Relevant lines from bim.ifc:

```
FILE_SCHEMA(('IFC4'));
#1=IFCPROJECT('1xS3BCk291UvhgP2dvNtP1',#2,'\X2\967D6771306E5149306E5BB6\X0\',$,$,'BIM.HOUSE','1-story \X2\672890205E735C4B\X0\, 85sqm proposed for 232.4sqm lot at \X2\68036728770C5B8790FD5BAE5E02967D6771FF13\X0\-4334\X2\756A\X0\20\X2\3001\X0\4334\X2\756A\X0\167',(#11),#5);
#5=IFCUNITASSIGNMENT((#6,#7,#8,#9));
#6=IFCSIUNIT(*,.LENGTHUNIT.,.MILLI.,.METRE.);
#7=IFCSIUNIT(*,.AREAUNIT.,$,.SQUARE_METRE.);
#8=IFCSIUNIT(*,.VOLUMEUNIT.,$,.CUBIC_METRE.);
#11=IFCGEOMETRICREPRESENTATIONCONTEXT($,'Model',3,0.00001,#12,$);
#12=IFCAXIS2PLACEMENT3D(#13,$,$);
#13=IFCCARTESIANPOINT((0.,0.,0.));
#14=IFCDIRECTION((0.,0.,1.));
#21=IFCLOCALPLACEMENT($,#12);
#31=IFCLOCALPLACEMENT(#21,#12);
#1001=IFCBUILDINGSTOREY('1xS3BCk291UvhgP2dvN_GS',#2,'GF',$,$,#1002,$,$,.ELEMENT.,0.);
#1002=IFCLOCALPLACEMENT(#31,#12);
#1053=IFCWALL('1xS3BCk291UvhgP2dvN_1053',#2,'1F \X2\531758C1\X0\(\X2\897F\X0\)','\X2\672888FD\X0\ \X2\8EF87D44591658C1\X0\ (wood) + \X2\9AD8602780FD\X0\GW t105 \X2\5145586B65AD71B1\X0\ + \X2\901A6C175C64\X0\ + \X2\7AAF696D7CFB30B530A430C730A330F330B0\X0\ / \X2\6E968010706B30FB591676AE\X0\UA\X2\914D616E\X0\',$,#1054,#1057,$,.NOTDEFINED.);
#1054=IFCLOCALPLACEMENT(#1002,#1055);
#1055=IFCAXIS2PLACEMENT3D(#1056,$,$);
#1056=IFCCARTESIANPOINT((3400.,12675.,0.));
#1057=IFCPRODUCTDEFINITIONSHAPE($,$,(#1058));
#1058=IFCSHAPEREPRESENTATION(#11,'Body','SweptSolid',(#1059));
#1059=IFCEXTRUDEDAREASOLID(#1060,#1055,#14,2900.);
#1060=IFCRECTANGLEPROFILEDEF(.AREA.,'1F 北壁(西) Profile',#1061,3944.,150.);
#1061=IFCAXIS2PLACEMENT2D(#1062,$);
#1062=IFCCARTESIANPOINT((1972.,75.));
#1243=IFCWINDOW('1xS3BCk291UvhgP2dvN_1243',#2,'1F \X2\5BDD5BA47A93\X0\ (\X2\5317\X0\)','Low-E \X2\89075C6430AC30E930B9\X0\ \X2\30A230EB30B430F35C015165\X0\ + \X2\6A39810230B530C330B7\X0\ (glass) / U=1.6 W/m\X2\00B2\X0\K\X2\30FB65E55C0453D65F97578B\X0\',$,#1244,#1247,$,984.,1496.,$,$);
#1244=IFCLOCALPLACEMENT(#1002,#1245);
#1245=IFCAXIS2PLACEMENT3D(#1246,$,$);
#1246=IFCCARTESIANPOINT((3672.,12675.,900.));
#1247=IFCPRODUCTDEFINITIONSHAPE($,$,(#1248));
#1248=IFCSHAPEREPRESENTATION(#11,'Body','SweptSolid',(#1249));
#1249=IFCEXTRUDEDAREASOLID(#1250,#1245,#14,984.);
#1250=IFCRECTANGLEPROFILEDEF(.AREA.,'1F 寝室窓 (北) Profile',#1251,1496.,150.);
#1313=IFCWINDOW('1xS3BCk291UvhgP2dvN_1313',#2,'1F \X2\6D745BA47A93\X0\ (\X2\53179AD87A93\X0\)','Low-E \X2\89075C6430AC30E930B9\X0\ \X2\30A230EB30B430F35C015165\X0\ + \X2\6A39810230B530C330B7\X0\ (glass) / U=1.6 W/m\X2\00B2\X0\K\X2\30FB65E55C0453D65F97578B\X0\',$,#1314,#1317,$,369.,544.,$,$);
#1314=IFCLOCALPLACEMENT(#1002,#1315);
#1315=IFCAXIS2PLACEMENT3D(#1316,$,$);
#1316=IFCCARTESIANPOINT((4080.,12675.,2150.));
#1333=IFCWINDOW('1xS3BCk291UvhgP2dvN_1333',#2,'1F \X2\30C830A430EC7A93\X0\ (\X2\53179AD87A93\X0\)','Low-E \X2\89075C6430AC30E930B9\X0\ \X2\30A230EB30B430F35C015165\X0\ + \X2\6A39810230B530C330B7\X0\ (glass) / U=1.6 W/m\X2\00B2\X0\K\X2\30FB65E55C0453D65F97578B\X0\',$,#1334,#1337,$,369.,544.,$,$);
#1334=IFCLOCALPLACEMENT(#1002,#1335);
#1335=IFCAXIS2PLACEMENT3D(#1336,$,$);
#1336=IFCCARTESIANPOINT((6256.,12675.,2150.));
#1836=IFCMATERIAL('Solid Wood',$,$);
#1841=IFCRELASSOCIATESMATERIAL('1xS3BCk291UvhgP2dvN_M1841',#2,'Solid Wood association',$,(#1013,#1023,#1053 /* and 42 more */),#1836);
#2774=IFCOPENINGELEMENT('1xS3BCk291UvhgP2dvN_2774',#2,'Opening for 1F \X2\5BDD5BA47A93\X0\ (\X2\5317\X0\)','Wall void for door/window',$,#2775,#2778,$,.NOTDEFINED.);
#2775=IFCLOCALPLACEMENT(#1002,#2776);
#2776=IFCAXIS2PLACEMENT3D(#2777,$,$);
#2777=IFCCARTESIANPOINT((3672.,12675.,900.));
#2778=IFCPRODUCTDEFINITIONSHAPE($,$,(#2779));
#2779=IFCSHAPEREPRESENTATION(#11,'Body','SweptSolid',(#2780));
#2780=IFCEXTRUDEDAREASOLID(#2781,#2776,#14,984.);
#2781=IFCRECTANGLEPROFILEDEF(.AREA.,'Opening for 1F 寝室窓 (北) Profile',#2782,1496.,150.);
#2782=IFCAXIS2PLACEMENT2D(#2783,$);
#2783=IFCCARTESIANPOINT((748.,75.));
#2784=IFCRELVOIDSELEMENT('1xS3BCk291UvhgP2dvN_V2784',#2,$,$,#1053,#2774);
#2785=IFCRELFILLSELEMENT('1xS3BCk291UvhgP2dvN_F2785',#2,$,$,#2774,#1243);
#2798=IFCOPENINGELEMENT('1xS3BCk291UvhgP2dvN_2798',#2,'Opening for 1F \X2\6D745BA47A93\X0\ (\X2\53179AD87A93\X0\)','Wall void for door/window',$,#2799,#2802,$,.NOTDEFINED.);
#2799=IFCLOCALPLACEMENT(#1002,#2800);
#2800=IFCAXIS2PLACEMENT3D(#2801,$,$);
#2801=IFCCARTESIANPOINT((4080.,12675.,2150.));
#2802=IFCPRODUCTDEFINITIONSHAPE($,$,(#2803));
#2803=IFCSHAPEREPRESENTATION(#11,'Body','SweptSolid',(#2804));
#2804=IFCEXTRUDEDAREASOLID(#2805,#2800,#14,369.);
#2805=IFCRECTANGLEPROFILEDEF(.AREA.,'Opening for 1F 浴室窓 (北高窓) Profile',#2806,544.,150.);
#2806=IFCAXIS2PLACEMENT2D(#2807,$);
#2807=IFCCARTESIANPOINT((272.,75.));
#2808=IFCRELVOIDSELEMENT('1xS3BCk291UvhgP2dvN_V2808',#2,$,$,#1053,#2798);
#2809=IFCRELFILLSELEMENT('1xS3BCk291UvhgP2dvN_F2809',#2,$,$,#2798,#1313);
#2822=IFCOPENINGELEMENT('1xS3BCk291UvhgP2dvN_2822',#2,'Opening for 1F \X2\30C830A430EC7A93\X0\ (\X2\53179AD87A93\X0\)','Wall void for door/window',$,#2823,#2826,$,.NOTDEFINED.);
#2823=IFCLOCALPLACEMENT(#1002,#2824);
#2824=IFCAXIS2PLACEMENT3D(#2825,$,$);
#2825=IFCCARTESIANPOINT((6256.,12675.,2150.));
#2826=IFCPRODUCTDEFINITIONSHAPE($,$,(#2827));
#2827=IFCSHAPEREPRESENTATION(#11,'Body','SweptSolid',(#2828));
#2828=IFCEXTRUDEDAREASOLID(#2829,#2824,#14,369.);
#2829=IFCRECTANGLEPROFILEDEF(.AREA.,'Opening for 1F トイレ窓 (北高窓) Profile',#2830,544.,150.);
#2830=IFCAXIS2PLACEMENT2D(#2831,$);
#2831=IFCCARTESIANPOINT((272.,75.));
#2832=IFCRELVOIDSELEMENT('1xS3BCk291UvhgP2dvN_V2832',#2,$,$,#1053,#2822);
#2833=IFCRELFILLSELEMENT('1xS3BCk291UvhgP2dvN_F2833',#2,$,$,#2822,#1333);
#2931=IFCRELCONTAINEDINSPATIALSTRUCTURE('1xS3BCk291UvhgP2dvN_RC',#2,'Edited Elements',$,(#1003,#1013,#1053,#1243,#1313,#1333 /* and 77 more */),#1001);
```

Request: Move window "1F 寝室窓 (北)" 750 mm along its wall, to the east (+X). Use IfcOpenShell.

```python
import ifcopenshell
import ifcopenshell.api.geometry
import ifcopenshell.util.placement
import ifcopenshell.util.unit

model = ifcopenshell.open("bim.ifc")
unit_scale = ifcopenshell.util.unit.calculate_unit_scale(model)

window = model.by_guid("1xS3BCk291UvhgP2dvN_1243")
opening = window.FillsVoids[0].RelatingOpeningElement
wall = opening.VoidsElements[0].RelatingBuildingElement

wall_matrix = ifcopenshell.util.placement.get_local_placement(wall.ObjectPlacement)
shift = wall_matrix[:3, 0] * 0.75 / unit_scale
before = ifcopenshell.util.placement.get_local_placement(window.ObjectPlacement)[:3, 3].copy()

# The window is not placed relative to its opening, so move both.
for product in (opening, window):
    matrix = ifcopenshell.util.placement.get_local_placement(product.ObjectPlacement)
    matrix[:3, 3] += shift
    ifcopenshell.api.geometry.edit_object_placement(model, product=product, matrix=matrix, is_si=False)

after = ifcopenshell.util.placement.get_local_placement(window.ObjectPlacement)[:3, 3]
print("window moved by", (after - before).round(3) + 0.0)

model.write("bim_v2.ifc")
```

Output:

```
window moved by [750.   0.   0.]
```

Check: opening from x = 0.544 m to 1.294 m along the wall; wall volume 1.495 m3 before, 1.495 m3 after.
